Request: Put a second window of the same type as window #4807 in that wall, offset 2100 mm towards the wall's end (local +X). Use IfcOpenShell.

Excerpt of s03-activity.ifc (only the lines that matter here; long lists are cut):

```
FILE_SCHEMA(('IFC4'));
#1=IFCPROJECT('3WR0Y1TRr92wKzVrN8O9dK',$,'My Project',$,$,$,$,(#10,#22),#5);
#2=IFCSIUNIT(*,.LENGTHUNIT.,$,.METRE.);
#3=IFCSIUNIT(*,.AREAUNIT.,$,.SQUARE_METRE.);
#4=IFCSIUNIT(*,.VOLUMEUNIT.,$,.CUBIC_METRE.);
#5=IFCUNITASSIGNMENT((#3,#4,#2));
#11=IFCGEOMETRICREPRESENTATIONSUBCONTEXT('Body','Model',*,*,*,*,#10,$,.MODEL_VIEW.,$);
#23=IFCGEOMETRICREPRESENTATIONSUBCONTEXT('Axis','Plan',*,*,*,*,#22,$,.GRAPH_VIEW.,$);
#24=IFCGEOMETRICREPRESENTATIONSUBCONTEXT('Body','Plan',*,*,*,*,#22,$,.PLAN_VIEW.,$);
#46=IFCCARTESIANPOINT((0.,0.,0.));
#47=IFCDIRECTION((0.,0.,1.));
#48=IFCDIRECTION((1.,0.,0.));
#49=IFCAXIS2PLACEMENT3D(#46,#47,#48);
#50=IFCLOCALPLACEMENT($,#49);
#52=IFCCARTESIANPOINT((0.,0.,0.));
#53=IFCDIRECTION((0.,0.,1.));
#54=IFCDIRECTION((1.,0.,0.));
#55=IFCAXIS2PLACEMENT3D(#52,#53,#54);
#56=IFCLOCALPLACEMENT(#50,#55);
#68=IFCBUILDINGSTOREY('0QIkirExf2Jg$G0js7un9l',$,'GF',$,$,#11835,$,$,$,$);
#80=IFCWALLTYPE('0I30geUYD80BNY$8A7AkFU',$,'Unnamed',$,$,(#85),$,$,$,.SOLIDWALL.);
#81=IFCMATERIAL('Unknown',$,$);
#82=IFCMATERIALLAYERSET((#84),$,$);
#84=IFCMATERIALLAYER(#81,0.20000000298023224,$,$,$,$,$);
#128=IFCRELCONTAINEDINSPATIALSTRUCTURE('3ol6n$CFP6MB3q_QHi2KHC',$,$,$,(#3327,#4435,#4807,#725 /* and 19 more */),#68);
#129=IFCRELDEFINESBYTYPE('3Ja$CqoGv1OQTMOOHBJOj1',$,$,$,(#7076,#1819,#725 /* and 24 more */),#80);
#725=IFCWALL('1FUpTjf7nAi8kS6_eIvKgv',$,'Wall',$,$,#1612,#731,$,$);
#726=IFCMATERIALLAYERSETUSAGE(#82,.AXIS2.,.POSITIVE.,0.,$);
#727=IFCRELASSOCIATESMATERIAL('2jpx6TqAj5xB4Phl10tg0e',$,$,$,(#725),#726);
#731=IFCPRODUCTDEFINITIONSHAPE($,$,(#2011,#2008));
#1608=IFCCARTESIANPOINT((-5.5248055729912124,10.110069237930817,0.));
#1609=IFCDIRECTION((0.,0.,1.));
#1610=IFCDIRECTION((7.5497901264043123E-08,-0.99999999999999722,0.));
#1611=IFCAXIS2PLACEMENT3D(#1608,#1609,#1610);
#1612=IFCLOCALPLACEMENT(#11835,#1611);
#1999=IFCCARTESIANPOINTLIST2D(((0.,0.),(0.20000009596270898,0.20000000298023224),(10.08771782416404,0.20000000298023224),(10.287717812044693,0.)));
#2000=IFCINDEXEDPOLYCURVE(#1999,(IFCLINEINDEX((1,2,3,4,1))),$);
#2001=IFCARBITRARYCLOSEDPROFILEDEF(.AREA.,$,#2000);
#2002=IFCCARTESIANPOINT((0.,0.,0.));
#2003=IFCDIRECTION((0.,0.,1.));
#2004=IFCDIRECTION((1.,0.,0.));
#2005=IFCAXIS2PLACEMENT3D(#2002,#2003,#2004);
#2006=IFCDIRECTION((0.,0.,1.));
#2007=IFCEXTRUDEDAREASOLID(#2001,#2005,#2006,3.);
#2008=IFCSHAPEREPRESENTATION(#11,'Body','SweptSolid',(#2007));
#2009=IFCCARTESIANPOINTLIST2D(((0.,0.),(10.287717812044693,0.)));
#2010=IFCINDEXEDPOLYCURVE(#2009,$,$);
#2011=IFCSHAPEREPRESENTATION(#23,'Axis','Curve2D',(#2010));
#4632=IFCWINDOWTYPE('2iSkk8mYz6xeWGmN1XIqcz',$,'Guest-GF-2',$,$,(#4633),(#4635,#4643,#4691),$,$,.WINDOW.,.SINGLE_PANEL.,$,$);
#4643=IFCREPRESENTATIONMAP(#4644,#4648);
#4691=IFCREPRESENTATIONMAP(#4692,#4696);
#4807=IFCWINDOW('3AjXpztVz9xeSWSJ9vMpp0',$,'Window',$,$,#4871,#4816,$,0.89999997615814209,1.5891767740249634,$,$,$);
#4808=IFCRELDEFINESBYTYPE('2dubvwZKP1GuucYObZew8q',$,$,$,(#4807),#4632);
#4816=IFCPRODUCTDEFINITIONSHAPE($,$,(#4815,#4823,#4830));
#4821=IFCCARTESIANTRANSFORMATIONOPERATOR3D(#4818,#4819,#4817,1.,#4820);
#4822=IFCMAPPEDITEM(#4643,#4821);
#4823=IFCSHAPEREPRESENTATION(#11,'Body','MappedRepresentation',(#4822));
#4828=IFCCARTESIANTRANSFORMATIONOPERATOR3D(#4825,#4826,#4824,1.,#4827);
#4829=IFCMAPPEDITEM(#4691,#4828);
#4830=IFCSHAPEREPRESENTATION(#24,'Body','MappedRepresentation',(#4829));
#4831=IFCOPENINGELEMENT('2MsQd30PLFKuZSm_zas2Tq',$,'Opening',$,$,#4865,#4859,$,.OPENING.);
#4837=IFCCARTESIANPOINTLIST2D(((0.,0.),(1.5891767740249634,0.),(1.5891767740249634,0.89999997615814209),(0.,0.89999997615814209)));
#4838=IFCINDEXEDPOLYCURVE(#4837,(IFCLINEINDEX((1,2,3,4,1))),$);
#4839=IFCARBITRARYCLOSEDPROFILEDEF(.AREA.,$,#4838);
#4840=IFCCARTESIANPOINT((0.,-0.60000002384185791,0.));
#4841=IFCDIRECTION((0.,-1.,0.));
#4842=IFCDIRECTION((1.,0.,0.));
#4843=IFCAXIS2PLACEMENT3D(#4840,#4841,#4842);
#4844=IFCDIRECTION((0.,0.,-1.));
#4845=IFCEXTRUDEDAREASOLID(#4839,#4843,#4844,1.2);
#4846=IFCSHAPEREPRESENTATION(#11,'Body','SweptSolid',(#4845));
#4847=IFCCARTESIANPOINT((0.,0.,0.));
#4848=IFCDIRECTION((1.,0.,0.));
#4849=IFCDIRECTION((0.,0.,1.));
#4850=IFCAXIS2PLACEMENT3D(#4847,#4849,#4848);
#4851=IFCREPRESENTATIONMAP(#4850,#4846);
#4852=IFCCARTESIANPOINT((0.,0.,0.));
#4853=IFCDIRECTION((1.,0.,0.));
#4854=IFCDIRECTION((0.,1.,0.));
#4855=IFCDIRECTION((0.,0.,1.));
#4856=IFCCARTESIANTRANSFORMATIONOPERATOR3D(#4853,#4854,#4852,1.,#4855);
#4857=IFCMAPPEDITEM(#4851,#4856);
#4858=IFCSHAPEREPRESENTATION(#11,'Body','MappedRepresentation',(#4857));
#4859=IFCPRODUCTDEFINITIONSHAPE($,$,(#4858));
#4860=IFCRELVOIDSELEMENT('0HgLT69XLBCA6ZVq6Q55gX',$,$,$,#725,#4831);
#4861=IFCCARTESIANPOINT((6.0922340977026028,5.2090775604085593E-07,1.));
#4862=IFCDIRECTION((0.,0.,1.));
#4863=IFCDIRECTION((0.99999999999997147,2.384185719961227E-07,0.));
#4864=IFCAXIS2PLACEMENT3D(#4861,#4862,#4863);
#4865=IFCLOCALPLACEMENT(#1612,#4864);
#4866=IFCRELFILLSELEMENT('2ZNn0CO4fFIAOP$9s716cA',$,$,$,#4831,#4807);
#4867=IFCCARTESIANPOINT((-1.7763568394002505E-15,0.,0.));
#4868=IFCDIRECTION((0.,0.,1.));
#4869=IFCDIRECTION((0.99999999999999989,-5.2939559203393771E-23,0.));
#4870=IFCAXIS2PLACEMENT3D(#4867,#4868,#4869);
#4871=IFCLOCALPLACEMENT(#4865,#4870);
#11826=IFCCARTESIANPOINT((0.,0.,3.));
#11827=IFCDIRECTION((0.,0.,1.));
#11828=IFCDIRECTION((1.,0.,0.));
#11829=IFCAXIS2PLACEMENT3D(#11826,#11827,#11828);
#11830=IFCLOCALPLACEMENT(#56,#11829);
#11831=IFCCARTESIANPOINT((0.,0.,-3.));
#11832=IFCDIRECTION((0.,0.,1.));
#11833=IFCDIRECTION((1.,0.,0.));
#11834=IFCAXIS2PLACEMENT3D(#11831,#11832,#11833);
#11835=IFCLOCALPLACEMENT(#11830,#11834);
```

```python
import ifcopenshell
import ifcopenshell.api.feature
import ifcopenshell.api.geometry
import ifcopenshell.api.root
import ifcopenshell.geom
import ifcopenshell.util.element
import ifcopenshell.util.placement
import ifcopenshell.util.shape
import ifcopenshell.util.unit

model = ifcopenshell.open("s03-activity.ifc")
unit_scale = ifcopenshell.util.unit.calculate_unit_scale(model)
settings = ifcopenshell.geom.settings()


def volume(element):
    """Net volume in cubic metres, openings subtracted."""
    shape = ifcopenshell.geom.create_shape(settings, element)
    return ifcopenshell.util.shape.get_volume(shape.geometry)


window = model.by_id(4807)
opening = window.FillsVoids[0].RelatingOpeningElement
wall = opening.VoidsElements[0].RelatingBuildingElement
before = volume(wall)
shift = ifcopenshell.util.placement.get_local_placement(wall.ObjectPlacement)[:3, 0] * 2.1 / unit_scale

# copy_class copies the void relationship, type, container and properties, but no geometry.
new_opening = ifcopenshell.api.root.copy_class(model, product=opening)
new_opening.Representation = ifcopenshell.util.element.copy_deep(
    model, opening.Representation, exclude=["IfcGeometricRepresentationContext", "IfcRepresentationMap"]
)
new_window = ifcopenshell.api.root.copy_class(model, product=window)
new_window.Representation = ifcopenshell.util.element.copy_deep(
    model, window.Representation, exclude=["IfcGeometricRepresentationContext", "IfcRepresentationMap"]
)
ifcopenshell.api.feature.add_filling(model, opening=new_opening, element=new_window)

for old, new in ((opening, new_opening), (window, new_window)):
    matrix = ifcopenshell.util.placement.get_local_placement(old.ObjectPlacement)
    matrix[:3, 3] += shift
    ifcopenshell.api.geometry.edit_object_placement(model, product=new, matrix=matrix, is_si=False)

after = volume(wall)

print(f"wall volume {before:.3f} -> {after:.3f} m3")

model.write("s03-activity-out.ifc")
```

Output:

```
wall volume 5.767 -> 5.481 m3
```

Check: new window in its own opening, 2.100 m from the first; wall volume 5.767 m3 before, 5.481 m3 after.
